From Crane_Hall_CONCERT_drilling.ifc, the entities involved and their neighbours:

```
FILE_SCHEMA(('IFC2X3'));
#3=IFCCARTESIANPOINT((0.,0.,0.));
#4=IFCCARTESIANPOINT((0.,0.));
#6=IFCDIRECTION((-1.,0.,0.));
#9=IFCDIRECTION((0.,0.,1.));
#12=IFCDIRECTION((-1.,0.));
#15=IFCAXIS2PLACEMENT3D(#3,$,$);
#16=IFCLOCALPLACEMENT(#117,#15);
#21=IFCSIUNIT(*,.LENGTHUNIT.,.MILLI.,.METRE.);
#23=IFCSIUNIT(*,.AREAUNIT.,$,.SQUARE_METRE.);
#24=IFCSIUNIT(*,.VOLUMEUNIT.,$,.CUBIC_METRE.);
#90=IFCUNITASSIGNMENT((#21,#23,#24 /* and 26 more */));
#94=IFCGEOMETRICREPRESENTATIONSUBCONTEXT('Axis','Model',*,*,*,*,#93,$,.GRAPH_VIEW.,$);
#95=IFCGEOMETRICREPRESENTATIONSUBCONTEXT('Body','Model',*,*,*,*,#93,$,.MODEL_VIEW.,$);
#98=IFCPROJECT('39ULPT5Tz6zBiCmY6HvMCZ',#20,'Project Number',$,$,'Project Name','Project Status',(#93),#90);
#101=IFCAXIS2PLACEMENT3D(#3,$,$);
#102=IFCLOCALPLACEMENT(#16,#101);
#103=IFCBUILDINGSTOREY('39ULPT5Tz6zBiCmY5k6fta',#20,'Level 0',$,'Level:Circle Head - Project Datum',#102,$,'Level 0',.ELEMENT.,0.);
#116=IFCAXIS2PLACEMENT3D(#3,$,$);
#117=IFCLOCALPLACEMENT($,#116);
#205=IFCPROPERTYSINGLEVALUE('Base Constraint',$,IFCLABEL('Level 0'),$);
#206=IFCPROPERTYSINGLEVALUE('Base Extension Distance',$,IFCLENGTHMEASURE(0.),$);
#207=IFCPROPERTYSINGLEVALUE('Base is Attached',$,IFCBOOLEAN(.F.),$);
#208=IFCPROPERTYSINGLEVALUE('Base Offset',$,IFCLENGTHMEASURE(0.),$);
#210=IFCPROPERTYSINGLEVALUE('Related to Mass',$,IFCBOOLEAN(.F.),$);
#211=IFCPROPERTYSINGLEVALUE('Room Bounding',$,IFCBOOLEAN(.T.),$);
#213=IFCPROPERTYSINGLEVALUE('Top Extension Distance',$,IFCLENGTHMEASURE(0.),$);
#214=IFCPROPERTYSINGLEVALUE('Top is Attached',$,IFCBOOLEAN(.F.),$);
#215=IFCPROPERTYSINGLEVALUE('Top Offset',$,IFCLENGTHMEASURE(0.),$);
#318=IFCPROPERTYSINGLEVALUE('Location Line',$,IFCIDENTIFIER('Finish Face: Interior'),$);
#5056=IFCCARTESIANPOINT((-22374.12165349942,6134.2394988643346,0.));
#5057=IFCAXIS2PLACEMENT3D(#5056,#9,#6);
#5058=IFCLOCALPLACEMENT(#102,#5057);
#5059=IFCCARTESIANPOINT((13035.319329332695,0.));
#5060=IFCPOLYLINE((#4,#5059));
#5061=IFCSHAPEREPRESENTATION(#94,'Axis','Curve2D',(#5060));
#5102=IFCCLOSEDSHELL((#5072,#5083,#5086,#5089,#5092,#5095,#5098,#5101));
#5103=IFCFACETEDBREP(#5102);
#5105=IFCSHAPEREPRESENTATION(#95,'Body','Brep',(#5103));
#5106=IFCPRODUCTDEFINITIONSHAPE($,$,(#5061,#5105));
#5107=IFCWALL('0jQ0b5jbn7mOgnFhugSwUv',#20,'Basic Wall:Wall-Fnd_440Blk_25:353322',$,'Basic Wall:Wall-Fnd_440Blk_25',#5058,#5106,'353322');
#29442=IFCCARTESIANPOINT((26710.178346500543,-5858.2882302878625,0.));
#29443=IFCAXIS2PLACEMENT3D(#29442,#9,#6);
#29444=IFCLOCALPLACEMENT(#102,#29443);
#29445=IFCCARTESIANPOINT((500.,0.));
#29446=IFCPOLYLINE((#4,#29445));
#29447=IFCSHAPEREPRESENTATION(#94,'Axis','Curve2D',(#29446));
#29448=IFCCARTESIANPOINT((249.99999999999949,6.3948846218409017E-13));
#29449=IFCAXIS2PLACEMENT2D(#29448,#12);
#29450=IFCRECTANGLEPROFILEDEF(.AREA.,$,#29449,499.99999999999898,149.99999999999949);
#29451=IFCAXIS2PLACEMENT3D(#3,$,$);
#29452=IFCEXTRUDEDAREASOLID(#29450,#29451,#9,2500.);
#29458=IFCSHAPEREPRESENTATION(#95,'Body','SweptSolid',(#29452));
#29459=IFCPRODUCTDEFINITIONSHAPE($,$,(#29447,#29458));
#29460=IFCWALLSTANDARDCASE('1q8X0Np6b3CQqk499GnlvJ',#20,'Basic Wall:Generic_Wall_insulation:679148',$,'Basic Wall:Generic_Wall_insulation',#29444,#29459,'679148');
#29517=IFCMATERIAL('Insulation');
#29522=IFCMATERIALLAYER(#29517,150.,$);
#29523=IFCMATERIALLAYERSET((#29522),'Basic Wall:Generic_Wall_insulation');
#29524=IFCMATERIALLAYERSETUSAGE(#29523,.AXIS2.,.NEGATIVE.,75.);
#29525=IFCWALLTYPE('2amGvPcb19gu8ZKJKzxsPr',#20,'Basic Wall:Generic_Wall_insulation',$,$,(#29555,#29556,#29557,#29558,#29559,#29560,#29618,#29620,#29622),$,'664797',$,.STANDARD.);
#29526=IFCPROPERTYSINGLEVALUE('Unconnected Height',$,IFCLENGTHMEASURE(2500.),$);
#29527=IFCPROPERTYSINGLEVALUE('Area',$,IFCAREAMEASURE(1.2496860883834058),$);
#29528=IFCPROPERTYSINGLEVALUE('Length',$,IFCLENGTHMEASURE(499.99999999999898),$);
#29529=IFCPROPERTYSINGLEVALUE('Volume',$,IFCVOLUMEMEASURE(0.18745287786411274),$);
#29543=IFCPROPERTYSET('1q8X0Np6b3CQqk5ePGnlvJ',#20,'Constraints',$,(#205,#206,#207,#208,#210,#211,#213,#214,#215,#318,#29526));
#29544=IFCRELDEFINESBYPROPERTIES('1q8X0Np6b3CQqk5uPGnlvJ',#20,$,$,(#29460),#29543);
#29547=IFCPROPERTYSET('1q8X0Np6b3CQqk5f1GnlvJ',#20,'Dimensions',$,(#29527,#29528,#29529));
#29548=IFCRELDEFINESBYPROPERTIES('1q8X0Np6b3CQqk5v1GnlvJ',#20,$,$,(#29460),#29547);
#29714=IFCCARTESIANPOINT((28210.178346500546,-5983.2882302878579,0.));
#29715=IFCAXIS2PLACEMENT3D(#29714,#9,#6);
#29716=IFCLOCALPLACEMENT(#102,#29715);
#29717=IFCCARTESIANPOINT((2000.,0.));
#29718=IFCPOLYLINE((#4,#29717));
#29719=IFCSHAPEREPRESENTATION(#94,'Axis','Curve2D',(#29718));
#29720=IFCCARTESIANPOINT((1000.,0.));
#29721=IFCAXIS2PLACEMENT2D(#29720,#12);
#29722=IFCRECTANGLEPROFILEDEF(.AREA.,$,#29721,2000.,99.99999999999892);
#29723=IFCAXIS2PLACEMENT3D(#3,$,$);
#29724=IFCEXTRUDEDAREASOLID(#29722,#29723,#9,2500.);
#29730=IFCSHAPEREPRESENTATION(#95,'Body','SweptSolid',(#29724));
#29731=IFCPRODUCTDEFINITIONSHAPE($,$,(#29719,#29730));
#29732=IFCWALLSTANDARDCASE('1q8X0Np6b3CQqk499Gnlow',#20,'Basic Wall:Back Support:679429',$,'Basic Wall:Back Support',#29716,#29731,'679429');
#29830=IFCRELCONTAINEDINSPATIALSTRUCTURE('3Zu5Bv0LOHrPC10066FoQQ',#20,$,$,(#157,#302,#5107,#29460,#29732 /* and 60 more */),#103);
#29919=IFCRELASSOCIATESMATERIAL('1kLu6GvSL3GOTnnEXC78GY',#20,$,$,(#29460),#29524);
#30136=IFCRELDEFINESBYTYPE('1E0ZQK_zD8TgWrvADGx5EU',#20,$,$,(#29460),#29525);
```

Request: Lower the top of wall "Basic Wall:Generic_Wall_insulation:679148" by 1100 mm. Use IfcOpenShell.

```python
import ifcopenshell
import ifcopenshell.api.pset
import ifcopenshell.geom
import ifcopenshell.util.element
import ifcopenshell.util.representation
import ifcopenshell.util.shape
import ifcopenshell.util.unit

model = ifcopenshell.open("Crane_Hall_CONCERT_drilling.ifc")
unit_scale = ifcopenshell.util.unit.calculate_unit_scale(model)
area_scale = ifcopenshell.util.unit.calculate_unit_scale(model, "AREAUNIT")
volume_scale = ifcopenshell.util.unit.calculate_unit_scale(model, "VOLUMEUNIT")
settings = ifcopenshell.geom.settings()


def volume(element):
    """Net volume in cubic metres, openings subtracted."""
    shape = ifcopenshell.geom.create_shape(settings, element)
    return ifcopenshell.util.shape.get_volume(shape.geometry)


wall = model.by_guid("1q8X0Np6b3CQqk499GnlvJ")
before = volume(wall)

body = ifcopenshell.util.representation.get_representation(wall, "Model", "Body")
solid = body.Items[0]
old_height = solid.Depth
solid.Depth -= 1.1 / unit_scale
after = volume(wall)
thickness = 0.15  # wall thickness in metres

# Update the stored height, areas and volumes.
pset = model.by_id(ifcopenshell.util.element.get_pset(wall, "Constraints", should_inherit=False)["id"])
ifcopenshell.api.pset.edit_pset(model, pset=pset, properties={
    "Unconnected Height": model.create_entity("IfcLengthMeasure", solid.Depth),
})
pset = model.by_id(ifcopenshell.util.element.get_pset(wall, "Dimensions", should_inherit=False)["id"])
ifcopenshell.api.pset.edit_pset(model, pset=pset, properties={
    "Area": model.create_entity("IfcAreaMeasure", after / thickness / area_scale),
    "Volume": model.create_entity("IfcVolumeMeasure", after / volume_scale),
})

print(f"height {old_height:g} -> {solid.Depth:g}, volume {before:.3f} -> {after:.3f} m3")

model.write("Crane_Hall_CONCERT_drilling_rev.ifc")
```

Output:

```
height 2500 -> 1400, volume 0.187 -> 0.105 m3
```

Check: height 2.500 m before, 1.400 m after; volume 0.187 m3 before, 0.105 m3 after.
